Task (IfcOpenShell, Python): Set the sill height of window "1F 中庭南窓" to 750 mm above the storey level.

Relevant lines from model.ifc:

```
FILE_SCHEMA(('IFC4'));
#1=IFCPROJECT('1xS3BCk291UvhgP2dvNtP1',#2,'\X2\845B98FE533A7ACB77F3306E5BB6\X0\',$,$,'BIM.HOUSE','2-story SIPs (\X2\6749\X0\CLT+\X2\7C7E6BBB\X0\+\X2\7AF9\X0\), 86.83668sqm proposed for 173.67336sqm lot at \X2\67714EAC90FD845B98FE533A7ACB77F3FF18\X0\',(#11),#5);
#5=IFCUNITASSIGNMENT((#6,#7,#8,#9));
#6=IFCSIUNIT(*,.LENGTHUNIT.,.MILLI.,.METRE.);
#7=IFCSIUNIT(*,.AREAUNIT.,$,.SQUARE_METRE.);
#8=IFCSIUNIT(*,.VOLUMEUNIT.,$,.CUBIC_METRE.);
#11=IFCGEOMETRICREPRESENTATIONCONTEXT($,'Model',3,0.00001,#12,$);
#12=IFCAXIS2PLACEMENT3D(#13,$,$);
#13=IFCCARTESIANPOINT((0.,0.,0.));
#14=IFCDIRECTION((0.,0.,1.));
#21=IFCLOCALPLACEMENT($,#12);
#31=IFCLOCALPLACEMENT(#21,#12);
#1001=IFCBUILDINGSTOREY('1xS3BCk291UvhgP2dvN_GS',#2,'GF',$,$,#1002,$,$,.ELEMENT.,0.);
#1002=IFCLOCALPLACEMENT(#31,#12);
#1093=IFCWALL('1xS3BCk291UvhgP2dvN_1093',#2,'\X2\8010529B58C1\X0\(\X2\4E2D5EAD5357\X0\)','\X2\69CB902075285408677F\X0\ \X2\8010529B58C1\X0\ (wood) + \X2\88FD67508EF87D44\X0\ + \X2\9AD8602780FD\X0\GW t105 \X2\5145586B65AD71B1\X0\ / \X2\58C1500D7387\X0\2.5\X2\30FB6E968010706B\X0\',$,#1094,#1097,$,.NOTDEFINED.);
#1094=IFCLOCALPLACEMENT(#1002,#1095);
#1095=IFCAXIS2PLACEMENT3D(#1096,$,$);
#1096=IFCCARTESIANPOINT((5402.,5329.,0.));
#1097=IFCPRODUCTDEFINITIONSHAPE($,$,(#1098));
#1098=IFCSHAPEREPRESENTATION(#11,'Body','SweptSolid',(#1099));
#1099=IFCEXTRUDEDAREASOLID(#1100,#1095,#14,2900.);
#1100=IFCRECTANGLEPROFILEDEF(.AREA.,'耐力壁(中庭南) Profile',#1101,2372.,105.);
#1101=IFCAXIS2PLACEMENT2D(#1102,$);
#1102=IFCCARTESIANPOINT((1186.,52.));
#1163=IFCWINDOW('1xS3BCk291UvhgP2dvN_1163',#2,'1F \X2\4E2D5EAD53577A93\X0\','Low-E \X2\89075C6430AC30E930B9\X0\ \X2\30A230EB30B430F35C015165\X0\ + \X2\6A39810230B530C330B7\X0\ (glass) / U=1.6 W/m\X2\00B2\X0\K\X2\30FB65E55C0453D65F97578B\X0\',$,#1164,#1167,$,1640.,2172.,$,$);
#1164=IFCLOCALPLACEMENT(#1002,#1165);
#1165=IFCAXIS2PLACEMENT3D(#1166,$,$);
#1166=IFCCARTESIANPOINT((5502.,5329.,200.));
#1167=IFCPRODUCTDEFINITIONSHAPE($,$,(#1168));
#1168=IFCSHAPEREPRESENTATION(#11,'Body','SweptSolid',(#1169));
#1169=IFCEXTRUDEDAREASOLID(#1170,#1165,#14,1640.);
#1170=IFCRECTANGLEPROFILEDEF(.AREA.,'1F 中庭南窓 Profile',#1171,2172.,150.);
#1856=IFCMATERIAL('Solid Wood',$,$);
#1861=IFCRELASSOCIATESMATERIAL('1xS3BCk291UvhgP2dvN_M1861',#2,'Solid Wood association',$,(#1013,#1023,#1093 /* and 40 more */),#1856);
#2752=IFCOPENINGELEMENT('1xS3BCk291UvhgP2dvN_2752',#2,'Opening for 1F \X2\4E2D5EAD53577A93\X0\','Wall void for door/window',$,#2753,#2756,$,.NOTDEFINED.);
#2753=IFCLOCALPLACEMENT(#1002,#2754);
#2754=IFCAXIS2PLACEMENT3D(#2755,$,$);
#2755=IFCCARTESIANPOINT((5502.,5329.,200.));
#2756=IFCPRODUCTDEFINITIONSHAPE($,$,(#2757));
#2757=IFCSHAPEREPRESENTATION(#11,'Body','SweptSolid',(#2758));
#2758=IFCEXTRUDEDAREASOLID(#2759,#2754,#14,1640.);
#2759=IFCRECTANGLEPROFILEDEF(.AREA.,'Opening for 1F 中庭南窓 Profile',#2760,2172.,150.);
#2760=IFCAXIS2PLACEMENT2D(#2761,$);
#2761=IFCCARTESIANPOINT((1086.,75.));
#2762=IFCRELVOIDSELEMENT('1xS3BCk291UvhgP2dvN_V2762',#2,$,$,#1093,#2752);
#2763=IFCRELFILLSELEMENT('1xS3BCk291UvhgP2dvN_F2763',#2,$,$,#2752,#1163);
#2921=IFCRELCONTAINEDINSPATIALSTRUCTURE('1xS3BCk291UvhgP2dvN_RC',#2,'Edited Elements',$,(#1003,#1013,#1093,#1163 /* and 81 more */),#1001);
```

```python
import numpy as np
import ifcopenshell
import ifcopenshell.api.geometry
import ifcopenshell.geom
import ifcopenshell.util.element
import ifcopenshell.util.placement
import ifcopenshell.util.shape
import ifcopenshell.util.unit

model = ifcopenshell.open("model.ifc")
unit_scale = ifcopenshell.util.unit.calculate_unit_scale(model)

window = model.by_guid("1xS3BCk291UvhgP2dvN_1163")
opening = window.FillsVoids[0].RelatingOpeningElement
storey = ifcopenshell.util.element.get_container(window, ifc_class="IfcBuildingStorey")
level = ifcopenshell.util.placement.get_local_placement(storey.ObjectPlacement)[2, 3]

# The opening's origin need not be at the sill, so measure its lowest point.
shape = ifcopenshell.geom.create_shape(ifcopenshell.geom.settings(), opening)
bottom = ifcopenshell.util.shape.get_shape_bottom_elevation(shape, shape.geometry) / unit_scale
dz = level + 750.0 - bottom

shift = np.array([0.0, 0.0, dz])
# The window is not placed relative to its opening, so move both.
for product in (opening, window):
    matrix = ifcopenshell.util.placement.get_local_placement(product.ObjectPlacement)
    matrix[:3, 3] += shift
    ifcopenshell.api.geometry.edit_object_placement(model, product=product, matrix=matrix, is_si=False)

print(f"moved by {dz * unit_scale:+.3f} m")

model.write("model_rev.ifc")
```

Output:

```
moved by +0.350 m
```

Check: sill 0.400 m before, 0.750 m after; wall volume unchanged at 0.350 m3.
